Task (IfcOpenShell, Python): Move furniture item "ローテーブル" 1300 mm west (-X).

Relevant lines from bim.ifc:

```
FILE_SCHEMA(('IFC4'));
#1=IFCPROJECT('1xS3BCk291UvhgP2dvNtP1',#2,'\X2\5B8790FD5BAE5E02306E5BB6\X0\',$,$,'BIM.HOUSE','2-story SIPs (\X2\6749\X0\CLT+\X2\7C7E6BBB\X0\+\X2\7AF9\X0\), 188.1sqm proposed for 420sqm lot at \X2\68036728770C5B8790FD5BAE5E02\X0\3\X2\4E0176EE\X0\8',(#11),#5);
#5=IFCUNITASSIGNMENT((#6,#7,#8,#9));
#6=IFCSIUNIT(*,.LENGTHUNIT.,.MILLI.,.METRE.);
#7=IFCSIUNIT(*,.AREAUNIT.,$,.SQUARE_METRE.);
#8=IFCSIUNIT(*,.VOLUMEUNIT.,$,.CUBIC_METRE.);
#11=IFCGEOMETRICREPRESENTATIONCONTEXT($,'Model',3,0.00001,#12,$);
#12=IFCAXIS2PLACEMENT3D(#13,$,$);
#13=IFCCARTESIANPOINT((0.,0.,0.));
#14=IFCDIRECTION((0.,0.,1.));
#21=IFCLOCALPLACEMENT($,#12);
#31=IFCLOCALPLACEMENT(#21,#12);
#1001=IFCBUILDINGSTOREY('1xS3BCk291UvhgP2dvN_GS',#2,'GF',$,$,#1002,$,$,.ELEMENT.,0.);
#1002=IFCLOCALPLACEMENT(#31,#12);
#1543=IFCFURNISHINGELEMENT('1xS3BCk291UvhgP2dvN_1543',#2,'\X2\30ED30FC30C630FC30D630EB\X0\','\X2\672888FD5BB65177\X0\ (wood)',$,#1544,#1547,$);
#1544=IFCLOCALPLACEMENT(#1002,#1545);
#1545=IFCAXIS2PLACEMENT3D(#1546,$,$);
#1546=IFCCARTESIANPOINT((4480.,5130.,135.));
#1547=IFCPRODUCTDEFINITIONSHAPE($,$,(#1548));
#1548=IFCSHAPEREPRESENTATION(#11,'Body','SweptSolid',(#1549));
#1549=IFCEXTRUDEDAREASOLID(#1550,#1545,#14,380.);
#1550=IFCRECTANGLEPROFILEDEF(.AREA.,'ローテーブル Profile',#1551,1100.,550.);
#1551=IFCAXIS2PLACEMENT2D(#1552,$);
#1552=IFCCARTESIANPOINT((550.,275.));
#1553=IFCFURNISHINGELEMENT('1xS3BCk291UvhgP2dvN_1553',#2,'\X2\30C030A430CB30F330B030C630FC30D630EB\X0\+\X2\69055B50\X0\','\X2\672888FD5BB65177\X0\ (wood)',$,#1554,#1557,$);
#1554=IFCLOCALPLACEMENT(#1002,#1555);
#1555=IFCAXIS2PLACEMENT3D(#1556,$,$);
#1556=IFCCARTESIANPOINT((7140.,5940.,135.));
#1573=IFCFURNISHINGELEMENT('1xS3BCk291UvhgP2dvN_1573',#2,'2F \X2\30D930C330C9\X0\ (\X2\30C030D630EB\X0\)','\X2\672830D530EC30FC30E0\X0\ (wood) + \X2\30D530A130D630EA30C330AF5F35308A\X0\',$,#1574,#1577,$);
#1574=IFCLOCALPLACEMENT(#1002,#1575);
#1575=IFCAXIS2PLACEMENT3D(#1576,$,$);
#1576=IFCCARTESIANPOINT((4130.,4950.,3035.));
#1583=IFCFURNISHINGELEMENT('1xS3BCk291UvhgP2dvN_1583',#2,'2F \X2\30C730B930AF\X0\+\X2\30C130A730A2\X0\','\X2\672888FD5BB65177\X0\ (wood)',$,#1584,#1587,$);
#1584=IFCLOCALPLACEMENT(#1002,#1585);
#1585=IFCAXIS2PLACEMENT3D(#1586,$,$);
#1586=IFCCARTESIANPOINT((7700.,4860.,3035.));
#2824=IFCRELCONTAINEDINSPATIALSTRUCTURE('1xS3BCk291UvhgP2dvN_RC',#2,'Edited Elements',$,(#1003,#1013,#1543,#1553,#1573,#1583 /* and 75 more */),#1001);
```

```python
import ifcopenshell
import ifcopenshell.api.geometry
import ifcopenshell.util.placement
import ifcopenshell.util.unit

model = ifcopenshell.open("bim.ifc")
unit_scale = ifcopenshell.util.unit.calculate_unit_scale(model)

item = model.by_guid("1xS3BCk291UvhgP2dvN_1543")
matrix = ifcopenshell.util.placement.get_local_placement(item.ObjectPlacement)
matrix[0, 3] -= 1.3 / unit_scale
ifcopenshell.api.geometry.edit_object_placement(model, product=item, matrix=matrix, is_si=False)

print(ifcopenshell.util.placement.get_local_placement(item.ObjectPlacement).round(3) + 0.0)

model.write("bim_v2.ifc")
```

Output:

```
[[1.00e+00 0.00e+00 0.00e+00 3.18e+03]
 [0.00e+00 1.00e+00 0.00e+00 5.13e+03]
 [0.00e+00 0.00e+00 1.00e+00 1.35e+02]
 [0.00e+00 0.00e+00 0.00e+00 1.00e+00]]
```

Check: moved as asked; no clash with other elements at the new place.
